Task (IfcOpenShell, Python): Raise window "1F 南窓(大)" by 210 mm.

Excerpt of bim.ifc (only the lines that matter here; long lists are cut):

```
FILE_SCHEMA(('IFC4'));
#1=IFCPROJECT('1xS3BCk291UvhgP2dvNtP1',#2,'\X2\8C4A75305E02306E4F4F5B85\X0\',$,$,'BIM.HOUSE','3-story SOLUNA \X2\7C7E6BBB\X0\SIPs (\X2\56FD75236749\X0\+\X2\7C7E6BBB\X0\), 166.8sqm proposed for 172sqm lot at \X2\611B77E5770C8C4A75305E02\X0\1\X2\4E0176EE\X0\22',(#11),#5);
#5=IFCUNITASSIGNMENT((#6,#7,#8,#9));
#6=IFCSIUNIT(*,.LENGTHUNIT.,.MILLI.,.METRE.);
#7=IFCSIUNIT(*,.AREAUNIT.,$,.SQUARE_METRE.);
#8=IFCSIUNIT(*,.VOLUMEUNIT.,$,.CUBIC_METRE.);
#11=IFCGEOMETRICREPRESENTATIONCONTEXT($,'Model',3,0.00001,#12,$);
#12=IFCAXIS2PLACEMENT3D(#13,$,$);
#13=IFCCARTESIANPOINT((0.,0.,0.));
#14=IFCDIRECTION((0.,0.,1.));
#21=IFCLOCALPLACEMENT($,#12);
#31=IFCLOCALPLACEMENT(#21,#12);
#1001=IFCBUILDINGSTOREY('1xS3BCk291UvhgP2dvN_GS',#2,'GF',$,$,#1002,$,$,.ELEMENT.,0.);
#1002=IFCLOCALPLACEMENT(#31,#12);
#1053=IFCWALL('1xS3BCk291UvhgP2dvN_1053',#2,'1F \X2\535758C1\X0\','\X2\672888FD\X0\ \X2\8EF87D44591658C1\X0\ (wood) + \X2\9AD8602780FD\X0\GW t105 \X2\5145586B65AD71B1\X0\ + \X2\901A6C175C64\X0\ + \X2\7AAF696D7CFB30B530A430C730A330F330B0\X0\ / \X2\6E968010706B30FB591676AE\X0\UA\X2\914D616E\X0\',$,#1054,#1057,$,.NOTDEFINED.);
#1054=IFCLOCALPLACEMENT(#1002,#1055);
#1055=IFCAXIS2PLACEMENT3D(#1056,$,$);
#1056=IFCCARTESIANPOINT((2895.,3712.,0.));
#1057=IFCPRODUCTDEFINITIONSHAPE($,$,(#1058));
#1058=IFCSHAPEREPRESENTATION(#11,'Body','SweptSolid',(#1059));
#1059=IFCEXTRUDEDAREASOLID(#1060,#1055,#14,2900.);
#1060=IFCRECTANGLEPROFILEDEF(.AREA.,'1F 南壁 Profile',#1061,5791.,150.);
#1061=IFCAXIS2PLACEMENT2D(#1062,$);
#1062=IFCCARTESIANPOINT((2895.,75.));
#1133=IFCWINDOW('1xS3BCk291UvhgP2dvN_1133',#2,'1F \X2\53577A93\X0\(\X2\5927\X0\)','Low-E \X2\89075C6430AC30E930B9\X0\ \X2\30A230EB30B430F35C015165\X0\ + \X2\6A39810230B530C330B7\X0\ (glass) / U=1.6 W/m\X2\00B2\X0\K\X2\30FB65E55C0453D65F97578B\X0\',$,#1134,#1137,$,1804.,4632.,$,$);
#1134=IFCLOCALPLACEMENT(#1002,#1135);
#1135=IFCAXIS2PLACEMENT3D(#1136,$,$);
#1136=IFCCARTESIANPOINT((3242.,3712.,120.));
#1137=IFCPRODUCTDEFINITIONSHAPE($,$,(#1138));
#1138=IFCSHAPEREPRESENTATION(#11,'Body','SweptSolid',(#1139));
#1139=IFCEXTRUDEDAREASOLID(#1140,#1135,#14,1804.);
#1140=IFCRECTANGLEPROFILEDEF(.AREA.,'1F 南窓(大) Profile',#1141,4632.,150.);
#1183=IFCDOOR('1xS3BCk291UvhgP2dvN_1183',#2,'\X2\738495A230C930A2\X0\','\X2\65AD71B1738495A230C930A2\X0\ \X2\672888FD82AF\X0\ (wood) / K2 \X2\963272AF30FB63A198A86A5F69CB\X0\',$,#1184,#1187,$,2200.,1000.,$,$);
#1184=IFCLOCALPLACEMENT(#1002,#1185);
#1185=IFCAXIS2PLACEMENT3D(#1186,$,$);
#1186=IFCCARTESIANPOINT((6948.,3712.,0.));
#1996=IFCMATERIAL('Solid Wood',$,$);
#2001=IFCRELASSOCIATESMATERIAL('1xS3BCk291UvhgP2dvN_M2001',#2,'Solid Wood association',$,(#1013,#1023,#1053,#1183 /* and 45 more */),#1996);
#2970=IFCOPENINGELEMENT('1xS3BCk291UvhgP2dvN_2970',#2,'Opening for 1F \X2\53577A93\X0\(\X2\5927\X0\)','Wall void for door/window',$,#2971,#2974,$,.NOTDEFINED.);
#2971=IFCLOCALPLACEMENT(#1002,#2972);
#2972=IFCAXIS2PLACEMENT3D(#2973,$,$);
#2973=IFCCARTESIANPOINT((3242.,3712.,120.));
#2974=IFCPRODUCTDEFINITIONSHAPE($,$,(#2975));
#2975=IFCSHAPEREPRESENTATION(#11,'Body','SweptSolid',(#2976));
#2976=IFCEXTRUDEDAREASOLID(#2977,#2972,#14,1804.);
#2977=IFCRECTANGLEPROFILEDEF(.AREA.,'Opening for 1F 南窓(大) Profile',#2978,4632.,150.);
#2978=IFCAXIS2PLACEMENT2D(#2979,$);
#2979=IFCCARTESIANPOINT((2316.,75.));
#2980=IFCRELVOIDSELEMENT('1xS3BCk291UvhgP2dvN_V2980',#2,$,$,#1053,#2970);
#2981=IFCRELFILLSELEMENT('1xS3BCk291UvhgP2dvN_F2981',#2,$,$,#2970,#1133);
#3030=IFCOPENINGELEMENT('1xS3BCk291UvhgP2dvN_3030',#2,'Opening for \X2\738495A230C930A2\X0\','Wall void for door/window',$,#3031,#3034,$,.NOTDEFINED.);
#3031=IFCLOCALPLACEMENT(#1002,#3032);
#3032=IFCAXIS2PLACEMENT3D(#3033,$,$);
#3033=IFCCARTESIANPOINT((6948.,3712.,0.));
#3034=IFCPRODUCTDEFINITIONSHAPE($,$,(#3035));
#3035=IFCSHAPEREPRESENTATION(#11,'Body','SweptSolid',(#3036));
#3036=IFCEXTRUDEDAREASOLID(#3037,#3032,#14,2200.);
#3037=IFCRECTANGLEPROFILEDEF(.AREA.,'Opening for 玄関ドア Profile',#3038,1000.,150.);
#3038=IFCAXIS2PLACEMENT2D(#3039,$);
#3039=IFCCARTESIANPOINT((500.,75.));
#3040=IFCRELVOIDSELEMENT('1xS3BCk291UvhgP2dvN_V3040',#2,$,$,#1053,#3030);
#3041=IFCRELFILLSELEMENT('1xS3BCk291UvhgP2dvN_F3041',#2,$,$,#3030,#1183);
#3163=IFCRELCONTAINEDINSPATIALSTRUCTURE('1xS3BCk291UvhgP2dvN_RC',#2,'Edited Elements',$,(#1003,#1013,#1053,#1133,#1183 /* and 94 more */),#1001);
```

```python
import numpy as np
import ifcopenshell
import ifcopenshell.api.geometry
import ifcopenshell.util.placement
import ifcopenshell.util.unit

model = ifcopenshell.open("bim.ifc")
unit_scale = ifcopenshell.util.unit.calculate_unit_scale(model)

window = model.by_guid("1xS3BCk291UvhgP2dvN_1133")
opening = window.FillsVoids[0].RelatingOpeningElement
dz = 210.0

shift = np.array([0.0, 0.0, dz])
# The window is not placed relative to its opening, so move both.
for product in (opening, window):
    matrix = ifcopenshell.util.placement.get_local_placement(product.ObjectPlacement)
    matrix[:3, 3] += shift
    ifcopenshell.api.geometry.edit_object_placement(model, product=product, matrix=matrix, is_si=False)

print(f"moved by {dz * unit_scale:+.3f} m")

model.write("bim-out.ifc")
```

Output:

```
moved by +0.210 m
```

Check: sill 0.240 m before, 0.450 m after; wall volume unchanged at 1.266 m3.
